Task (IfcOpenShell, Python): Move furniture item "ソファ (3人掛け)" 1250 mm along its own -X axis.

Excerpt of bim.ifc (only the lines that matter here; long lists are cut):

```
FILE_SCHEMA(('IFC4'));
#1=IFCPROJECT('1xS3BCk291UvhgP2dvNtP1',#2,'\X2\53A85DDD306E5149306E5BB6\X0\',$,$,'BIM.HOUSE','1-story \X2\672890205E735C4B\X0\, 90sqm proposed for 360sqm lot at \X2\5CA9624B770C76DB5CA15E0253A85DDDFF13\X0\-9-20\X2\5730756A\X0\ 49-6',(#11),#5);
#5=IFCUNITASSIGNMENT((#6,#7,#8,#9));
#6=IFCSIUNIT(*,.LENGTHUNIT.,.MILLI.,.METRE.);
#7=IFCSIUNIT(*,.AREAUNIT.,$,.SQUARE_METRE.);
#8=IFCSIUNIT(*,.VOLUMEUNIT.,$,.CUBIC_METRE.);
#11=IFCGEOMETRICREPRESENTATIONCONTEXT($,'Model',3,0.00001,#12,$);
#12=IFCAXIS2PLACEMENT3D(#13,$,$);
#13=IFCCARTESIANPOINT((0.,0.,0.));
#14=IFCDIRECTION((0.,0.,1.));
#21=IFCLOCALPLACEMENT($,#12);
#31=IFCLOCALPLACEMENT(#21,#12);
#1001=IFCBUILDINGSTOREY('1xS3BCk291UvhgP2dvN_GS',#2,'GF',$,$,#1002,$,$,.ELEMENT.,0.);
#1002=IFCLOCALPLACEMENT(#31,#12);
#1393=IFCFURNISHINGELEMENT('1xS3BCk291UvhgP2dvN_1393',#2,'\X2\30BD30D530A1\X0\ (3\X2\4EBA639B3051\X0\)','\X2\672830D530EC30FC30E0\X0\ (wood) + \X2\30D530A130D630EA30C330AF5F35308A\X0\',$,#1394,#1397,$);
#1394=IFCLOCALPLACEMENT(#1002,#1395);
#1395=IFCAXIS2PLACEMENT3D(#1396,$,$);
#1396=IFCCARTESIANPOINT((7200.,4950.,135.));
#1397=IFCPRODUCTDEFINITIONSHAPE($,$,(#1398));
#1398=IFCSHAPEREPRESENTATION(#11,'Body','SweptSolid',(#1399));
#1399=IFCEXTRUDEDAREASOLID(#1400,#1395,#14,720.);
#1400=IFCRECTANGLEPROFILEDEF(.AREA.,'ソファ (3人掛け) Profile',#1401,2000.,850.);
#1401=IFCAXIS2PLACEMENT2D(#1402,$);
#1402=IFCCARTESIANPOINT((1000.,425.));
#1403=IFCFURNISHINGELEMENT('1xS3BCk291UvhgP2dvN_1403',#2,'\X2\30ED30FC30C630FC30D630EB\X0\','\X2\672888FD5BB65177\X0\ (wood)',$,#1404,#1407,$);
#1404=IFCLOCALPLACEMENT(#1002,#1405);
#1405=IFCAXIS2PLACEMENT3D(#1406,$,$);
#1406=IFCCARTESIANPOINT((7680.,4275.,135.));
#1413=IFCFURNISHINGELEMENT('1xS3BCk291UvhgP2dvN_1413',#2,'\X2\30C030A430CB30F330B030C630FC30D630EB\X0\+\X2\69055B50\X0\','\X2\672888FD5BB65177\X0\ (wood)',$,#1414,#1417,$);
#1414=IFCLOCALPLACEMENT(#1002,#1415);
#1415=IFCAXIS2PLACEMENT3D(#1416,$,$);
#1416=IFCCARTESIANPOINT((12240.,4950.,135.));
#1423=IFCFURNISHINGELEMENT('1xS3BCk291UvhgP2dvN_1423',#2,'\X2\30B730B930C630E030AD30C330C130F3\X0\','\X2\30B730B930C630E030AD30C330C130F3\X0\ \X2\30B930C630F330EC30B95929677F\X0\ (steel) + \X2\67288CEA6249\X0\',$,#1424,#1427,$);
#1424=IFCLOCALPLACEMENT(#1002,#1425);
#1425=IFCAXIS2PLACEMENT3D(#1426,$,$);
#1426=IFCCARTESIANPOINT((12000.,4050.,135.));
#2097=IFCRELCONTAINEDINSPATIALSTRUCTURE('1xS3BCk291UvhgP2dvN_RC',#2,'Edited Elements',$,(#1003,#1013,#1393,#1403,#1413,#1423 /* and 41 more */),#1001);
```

```python
import ifcopenshell
import ifcopenshell.api.geometry
import ifcopenshell.util.placement
import ifcopenshell.util.unit

model = ifcopenshell.open("bim.ifc")
unit_scale = ifcopenshell.util.unit.calculate_unit_scale(model)

item = model.by_id(1393)
matrix = ifcopenshell.util.placement.get_local_placement(item.ObjectPlacement)
matrix[:3, 3] -= matrix[:3, 0] * 1.25 / unit_scale
ifcopenshell.api.geometry.edit_object_placement(model, product=item, matrix=matrix, is_si=False)

print(ifcopenshell.util.placement.get_local_placement(item.ObjectPlacement).round(3) + 0.0)

model.write("bim_updated.ifc")
```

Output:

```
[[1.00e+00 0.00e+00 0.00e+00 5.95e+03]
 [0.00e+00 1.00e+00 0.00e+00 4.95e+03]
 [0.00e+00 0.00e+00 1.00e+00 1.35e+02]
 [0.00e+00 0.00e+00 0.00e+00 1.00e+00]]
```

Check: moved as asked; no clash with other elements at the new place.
